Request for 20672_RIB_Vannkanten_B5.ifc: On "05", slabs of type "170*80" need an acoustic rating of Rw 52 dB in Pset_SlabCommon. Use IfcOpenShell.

First a look at what the model holds.

```python
import ifcopenshell
import ifcopenshell.util.element

model = ifcopenshell.open("20672_RIB_Vannkanten_B5.ifc")
print(model.schema)
storey = next(s for s in model.by_type("IfcBuildingStorey") if s.Name == "05")
slabs = [e for e in ifcopenshell.util.element.get_decomposition(storey) if e.is_a("IfcSlab")]
seen = {}
for e in slabs:
    element_type = ifcopenshell.util.element.get_type(e)
    key = (element_type.Name if element_type != e and element_type else None, ifcopenshell.util.element.get_pset(e, "Pset_SlabCommon", "AcousticRating"))
    seen[key] = seen.get(key, 0) + 1
for (name, value), count in sorted(seen.items(), key=str):
    print(count, "x", name, "|", value)
```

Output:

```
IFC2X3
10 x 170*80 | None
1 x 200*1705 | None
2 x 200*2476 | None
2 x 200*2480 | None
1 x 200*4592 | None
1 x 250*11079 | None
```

```python
import ifcopenshell
import ifcopenshell.api.pset
import ifcopenshell.util.element

model = ifcopenshell.open("20672_RIB_Vannkanten_B5.ifc")

storey = next(s for s in model.by_type("IfcBuildingStorey") if s.Name == "05")
slabs = [e for e in ifcopenshell.util.element.get_decomposition(storey) if e.is_a("IfcSlab")]

count = 0
for e in slabs:
    element_type = ifcopenshell.util.element.get_type(e)
    if element_type in (None, e) or element_type.Name != "170*80":
        continue
    # add_pset returns the element's existing set when there is one.
    pset = ifcopenshell.api.pset.add_pset(model, product=e, name="Pset_SlabCommon")
    ifcopenshell.api.pset.edit_pset(model, pset=pset, properties={"AcousticRating": "Rw 52 dB"})
    count += 1

print(count, "slabs updated")

model.write("20672_RIB_Vannkanten_B5_rev.ifc")
```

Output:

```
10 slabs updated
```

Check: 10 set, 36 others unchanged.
